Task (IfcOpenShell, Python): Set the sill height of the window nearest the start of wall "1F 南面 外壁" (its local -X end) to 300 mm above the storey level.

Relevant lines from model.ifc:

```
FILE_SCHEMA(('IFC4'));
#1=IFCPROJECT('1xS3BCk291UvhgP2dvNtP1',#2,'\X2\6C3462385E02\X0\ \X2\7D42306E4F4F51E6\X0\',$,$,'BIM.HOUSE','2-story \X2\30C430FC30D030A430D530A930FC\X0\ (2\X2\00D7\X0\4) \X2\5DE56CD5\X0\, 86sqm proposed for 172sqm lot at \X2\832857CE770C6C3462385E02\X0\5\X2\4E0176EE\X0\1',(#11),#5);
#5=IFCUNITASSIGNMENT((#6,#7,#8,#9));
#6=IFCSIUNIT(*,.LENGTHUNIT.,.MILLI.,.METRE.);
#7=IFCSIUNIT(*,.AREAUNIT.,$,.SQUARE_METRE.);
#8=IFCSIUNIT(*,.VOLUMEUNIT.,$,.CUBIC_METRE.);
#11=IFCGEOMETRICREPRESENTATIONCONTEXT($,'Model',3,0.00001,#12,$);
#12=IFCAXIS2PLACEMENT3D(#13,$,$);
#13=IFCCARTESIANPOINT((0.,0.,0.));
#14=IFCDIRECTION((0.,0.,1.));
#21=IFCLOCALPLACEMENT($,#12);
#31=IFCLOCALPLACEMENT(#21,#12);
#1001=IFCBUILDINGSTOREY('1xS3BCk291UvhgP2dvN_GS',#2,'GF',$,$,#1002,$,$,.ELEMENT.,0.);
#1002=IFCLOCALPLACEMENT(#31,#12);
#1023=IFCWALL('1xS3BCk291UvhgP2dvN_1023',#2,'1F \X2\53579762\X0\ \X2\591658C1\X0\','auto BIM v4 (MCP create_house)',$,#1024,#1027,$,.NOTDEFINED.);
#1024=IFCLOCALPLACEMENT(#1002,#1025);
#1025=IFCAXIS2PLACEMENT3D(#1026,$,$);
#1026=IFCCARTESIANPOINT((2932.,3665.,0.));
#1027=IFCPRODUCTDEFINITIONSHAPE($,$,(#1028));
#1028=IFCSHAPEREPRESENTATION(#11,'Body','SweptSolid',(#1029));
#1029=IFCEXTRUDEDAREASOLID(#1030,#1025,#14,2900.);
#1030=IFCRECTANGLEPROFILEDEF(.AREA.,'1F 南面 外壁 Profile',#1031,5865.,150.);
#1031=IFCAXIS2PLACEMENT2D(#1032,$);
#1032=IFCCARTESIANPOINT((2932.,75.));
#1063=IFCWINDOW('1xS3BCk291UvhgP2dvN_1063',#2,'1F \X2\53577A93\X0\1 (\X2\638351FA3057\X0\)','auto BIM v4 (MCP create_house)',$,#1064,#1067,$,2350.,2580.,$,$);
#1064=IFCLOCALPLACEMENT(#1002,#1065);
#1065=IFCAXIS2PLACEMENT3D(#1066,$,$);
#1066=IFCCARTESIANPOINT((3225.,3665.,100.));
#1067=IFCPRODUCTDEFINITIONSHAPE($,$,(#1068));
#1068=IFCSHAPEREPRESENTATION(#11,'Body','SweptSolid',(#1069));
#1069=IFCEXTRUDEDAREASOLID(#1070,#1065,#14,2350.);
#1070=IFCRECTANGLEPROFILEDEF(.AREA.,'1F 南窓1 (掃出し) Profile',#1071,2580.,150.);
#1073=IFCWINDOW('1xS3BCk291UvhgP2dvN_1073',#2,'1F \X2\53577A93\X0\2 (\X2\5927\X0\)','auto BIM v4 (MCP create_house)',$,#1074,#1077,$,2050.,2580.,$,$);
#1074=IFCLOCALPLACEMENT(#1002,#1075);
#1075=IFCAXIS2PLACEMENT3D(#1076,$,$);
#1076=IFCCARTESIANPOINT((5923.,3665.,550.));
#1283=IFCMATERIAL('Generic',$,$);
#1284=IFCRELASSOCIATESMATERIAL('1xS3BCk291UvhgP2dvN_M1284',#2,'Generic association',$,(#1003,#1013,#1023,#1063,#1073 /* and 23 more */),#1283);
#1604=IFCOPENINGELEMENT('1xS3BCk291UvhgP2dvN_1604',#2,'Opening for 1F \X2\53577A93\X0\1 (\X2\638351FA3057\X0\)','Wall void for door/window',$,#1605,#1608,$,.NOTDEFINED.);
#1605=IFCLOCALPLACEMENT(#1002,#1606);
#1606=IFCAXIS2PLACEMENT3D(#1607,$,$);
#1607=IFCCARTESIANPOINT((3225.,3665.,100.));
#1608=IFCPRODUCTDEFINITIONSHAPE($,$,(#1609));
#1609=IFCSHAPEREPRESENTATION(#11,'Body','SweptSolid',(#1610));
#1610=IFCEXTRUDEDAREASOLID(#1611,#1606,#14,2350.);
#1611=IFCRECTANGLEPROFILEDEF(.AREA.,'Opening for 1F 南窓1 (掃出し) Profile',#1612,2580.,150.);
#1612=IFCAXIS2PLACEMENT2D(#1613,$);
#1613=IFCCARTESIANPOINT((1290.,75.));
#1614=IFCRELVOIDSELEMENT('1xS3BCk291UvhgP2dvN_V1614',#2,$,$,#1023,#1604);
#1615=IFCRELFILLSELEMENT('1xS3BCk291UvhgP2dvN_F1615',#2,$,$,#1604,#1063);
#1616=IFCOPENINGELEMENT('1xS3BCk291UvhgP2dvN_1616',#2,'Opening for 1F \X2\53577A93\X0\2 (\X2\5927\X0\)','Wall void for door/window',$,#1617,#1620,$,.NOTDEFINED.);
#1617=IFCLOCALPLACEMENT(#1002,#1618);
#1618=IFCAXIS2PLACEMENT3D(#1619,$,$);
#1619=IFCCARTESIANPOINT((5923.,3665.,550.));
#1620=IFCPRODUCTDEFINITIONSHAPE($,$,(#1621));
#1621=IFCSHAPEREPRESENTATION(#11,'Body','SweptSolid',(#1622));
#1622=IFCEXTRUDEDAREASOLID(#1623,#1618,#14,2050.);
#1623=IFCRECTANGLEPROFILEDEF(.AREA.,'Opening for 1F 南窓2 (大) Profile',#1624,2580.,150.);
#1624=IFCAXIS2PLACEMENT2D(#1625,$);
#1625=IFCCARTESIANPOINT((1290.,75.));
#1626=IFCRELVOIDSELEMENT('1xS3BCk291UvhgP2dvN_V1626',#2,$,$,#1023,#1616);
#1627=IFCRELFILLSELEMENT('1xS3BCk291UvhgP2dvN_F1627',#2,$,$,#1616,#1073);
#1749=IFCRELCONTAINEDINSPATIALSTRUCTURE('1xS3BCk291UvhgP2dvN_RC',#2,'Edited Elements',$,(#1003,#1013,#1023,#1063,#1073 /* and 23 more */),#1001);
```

```python
import numpy as np
import ifcopenshell
import ifcopenshell.api.geometry
import ifcopenshell.geom
import ifcopenshell.util.element
import ifcopenshell.util.placement
import ifcopenshell.util.shape
import ifcopenshell.util.unit

model = ifcopenshell.open("model.ifc")
unit_scale = ifcopenshell.util.unit.calculate_unit_scale(model)

window = model.by_guid("1xS3BCk291UvhgP2dvN_1063")
opening = window.FillsVoids[0].RelatingOpeningElement
storey = ifcopenshell.util.element.get_container(window, ifc_class="IfcBuildingStorey")
level = ifcopenshell.util.placement.get_local_placement(storey.ObjectPlacement)[2, 3]

# The opening's origin need not be at the sill, so measure its lowest point.
shape = ifcopenshell.geom.create_shape(ifcopenshell.geom.settings(), opening)
bottom = ifcopenshell.util.shape.get_shape_bottom_elevation(shape, shape.geometry) / unit_scale
dz = level + 0.3 / unit_scale - bottom

shift = np.array([0.0, 0.0, dz])
# The window is not placed relative to its opening, so move both.
for product in (opening, window):
    matrix = ifcopenshell.util.placement.get_local_placement(product.ObjectPlacement)
    matrix[:3, 3] += shift
    ifcopenshell.api.geometry.edit_object_placement(model, product=product, matrix=matrix, is_si=False)

print(f"moved by {dz * unit_scale:+.3f} m")

model.write("model_updated.ifc")
```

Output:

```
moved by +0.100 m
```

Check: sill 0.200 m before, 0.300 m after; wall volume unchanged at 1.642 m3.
